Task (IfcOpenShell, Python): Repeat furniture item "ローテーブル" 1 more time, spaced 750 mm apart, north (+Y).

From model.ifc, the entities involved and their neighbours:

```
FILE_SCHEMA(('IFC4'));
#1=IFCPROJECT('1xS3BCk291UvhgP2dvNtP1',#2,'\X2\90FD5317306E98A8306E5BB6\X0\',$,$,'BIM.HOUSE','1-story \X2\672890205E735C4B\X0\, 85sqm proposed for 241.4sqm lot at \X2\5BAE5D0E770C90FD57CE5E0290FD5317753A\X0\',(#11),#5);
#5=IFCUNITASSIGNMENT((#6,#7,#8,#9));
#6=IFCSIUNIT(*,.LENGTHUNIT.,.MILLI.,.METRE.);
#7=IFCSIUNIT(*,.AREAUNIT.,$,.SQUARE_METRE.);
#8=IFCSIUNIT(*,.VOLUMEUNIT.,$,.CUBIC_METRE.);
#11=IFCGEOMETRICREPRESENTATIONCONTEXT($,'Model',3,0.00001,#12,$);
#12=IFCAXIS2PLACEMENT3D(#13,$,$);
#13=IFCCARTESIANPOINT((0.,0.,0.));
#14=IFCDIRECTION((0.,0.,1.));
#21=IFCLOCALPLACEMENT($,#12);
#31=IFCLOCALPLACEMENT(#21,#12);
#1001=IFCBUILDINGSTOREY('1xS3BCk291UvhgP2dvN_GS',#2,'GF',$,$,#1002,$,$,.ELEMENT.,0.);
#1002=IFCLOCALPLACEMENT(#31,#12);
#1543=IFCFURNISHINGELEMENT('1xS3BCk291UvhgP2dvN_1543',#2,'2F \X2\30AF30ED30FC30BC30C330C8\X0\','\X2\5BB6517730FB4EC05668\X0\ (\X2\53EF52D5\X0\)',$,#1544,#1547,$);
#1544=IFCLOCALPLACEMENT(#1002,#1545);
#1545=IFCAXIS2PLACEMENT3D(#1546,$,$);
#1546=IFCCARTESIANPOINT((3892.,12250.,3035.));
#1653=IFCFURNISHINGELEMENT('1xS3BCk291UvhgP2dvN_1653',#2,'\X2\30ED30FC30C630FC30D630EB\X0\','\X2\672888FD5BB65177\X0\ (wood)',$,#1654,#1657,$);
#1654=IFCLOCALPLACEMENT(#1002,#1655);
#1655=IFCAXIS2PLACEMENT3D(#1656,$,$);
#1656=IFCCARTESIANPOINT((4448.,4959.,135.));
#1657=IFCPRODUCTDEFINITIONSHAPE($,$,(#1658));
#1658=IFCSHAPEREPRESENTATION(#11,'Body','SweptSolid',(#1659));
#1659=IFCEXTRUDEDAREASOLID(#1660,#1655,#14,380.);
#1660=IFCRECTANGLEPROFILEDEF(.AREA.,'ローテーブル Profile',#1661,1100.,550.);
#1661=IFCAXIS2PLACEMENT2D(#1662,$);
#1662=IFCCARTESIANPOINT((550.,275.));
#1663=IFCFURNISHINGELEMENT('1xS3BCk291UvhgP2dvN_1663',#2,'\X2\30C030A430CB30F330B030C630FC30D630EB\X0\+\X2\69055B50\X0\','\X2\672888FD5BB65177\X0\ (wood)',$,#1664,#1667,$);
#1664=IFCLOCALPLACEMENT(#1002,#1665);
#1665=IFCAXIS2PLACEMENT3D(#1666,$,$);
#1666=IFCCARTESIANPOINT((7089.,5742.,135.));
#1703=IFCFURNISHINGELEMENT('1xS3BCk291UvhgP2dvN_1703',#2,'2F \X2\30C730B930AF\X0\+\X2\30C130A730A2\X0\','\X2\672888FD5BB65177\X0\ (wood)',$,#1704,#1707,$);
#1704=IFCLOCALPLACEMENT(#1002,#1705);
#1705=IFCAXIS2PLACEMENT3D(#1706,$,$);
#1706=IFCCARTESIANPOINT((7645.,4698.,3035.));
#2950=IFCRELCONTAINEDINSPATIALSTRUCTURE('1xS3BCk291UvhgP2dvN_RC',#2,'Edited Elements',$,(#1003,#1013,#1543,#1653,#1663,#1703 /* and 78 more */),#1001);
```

```python
import numpy as np
import ifcopenshell
import ifcopenshell.api.geometry
import ifcopenshell.api.root
import ifcopenshell.util.element
import ifcopenshell.util.placement

model = ifcopenshell.open("model.ifc")


def reuse_history(source, copy):
    """copy_class also copies each property set's owner history, people and application; keep the originals."""
    for rel in copy.IsDefinedBy:
        if rel.is_a("IfcRelDefinesByProperties") and (history := rel.RelatingPropertyDefinition.OwnerHistory):
            rel.RelatingPropertyDefinition.OwnerHistory = source.OwnerHistory
            ifcopenshell.util.element.remove_deep2(model, history)


source = model.by_guid("1xS3BCk291UvhgP2dvN_1653")
base = ifcopenshell.util.placement.get_local_placement(source.ObjectPlacement)
step = np.array([0.0, 1.0, 0.0]) * 750.0

for i in range(1, 2):
    copy = ifcopenshell.api.root.copy_class(model, product=source)
    copy.Representation = ifcopenshell.util.element.copy_deep(
        model, source.Representation, exclude=["IfcGeometricRepresentationContext", "IfcRepresentationMap"]
    )
    reuse_history(source, copy)
    matrix = base.copy()
    matrix[:3, 3] += i * step
    print("added at", matrix[:3, 3].round(3) + 0.0)
    ifcopenshell.api.geometry.edit_object_placement(model, product=copy, matrix=matrix, is_si=False)

model.write("model_rev.ifc")
```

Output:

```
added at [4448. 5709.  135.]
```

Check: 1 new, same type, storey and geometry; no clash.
